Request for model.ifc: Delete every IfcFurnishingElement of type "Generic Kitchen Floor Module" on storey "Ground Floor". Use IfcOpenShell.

First a look at what the model holds.

```python
import ifcopenshell
import ifcopenshell.util.element

model = ifcopenshell.open("model.ifc")
print(model.schema)
storey = next(s for s in model.by_type("IfcBuildingStorey") if s.Name == "Ground Floor")
furniture = [e for e in ifcopenshell.util.element.get_decomposition(storey) if e.is_a("IfcFurnishingElement")]
seen = {}
for e in furniture:
    element_type = ifcopenshell.util.element.get_type(e)
    name = element_type.Name if element_type not in (None, e) else None
    seen[name] = seen.get(name, 0) + 1
for name, count in sorted(seen.items(), key=str):
    print(count, "x", name)
```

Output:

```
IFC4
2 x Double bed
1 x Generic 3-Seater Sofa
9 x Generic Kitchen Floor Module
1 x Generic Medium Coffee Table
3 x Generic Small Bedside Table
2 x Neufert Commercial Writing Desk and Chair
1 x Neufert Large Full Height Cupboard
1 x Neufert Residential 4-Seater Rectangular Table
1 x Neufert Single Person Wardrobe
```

```python
import ifcopenshell
import ifcopenshell.api.root
import ifcopenshell.util.element

model = ifcopenshell.open("model.ifc")

storey = next(s for s in model.by_type("IfcBuildingStorey") if s.Name == "Ground Floor")
furniture = [e for e in ifcopenshell.util.element.get_decomposition(storey) if e.is_a("IfcFurnishingElement")]
targets = [e for e in furniture if (t := ifcopenshell.util.element.get_type(e)) not in (None, e) and t.Name == "Generic Kitchen Floor Module"]

for e in targets:
    ifcopenshell.api.root.remove_product(model, product=e)
print(len(targets), "removed")

model.write("model_v2.ifc")
```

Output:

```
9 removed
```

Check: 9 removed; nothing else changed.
